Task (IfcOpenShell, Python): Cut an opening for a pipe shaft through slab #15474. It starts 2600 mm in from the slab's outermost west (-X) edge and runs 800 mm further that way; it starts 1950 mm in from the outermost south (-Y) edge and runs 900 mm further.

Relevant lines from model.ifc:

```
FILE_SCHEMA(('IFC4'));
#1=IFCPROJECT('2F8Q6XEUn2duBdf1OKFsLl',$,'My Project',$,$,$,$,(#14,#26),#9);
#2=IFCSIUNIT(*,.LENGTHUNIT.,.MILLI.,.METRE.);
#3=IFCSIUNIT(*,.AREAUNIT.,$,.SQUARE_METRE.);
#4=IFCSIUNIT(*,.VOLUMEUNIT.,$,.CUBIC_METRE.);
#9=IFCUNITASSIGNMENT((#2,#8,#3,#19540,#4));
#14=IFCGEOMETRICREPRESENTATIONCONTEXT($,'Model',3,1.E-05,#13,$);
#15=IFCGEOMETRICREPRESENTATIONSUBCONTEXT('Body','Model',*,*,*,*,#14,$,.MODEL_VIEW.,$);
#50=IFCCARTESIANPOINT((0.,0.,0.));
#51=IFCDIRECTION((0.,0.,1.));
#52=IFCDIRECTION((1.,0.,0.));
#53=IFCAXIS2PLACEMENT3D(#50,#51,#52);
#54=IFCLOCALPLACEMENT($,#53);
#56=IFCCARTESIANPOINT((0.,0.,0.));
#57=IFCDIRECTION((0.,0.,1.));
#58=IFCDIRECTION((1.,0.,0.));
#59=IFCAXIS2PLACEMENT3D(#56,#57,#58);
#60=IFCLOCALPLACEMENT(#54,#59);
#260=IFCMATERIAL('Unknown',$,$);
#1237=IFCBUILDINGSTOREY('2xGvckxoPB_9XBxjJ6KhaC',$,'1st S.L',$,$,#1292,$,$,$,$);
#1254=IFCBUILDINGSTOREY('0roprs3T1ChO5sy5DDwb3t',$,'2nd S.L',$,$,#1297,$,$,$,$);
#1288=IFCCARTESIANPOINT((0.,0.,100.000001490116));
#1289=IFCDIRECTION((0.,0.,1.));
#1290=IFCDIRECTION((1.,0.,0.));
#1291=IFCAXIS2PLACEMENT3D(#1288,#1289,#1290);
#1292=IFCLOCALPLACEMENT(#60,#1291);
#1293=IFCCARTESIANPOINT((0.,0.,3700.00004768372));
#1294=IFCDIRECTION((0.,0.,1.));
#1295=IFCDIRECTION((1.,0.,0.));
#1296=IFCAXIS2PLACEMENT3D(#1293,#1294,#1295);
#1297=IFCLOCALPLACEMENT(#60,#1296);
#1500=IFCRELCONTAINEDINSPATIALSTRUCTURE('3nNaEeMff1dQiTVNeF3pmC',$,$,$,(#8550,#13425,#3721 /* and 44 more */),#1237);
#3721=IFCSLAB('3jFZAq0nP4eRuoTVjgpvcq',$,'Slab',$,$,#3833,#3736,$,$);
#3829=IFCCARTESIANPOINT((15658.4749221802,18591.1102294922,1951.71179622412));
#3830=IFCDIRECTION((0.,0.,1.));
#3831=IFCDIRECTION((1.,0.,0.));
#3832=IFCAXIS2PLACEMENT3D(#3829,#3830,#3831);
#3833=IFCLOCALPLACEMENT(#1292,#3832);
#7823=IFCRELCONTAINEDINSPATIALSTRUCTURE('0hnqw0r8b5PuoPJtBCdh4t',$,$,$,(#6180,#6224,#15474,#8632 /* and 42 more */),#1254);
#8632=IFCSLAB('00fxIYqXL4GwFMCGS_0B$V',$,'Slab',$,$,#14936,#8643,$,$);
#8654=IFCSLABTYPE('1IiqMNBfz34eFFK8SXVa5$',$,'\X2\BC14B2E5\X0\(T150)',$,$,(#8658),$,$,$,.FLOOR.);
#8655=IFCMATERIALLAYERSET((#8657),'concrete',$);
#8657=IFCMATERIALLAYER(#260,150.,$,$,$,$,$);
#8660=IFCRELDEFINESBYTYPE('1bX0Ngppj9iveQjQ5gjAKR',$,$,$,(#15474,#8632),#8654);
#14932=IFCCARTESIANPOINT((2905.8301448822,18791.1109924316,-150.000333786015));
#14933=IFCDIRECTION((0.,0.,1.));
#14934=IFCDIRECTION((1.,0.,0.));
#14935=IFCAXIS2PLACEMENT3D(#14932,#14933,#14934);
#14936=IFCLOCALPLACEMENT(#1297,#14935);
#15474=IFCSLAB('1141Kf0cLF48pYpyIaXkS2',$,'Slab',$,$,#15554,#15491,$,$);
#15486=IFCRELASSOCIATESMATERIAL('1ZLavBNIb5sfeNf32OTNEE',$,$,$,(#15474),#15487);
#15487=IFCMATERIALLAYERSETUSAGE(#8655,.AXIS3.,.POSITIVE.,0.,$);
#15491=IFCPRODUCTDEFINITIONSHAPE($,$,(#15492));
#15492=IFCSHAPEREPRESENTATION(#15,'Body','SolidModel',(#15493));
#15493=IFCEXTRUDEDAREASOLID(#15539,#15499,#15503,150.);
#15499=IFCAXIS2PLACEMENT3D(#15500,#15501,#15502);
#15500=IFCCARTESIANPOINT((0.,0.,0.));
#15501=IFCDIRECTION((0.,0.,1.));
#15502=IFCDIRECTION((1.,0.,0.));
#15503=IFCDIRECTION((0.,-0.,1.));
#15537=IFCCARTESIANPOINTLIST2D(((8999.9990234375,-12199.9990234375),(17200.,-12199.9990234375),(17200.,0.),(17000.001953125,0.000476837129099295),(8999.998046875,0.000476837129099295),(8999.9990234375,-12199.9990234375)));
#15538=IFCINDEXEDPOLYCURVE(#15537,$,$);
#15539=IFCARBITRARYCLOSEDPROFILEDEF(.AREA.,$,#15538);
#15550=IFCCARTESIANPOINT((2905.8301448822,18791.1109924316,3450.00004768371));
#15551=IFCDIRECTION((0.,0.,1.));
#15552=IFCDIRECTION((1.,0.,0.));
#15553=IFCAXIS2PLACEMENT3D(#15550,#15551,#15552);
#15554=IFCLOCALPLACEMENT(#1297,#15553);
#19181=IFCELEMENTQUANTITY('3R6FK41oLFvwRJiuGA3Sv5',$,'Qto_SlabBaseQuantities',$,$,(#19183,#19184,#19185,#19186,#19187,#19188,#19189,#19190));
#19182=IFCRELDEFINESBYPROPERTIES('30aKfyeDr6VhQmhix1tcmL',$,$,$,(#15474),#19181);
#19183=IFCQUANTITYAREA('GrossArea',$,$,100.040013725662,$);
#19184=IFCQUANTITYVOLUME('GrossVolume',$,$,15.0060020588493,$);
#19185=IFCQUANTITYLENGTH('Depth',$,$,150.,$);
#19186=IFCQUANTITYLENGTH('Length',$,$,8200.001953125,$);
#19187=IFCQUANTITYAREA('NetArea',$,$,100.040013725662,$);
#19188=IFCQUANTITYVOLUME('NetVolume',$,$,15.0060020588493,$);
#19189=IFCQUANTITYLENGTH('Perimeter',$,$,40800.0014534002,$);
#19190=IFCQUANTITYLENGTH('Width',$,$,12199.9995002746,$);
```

```python
import numpy as np
import ifcopenshell
import ifcopenshell.api.feature
import ifcopenshell.api.geometry
import ifcopenshell.api.pset
import ifcopenshell.api.root
import ifcopenshell.geom
import ifcopenshell.util.element
import ifcopenshell.util.placement
import ifcopenshell.util.representation
import ifcopenshell.util.shape
import ifcopenshell.util.unit

model = ifcopenshell.open("model.ifc")
unit_scale = ifcopenshell.util.unit.calculate_unit_scale(model)
area_scale = ifcopenshell.util.unit.calculate_unit_scale(model, "AREAUNIT")
volume_scale = ifcopenshell.util.unit.calculate_unit_scale(model, "VOLUMEUNIT")
settings = ifcopenshell.geom.settings()


def volume(element):
    """Net volume in cubic metres, openings subtracted."""
    shape = ifcopenshell.geom.create_shape(settings, element)
    return ifcopenshell.util.shape.get_volume(shape.geometry)


slab = model.by_guid("1141Kf0cLF48pYpyIaXkS2")
before = volume(slab)

# Extent in the slab's own axes, in metres. The edges named are its -X and -Y sides.
slab_shape = ifcopenshell.geom.create_shape(settings, slab)
vertices = ifcopenshell.util.shape.get_vertices(slab_shape.geometry)
x_min, y_min, bottom = vertices.min(axis=0)
top = vertices[:, 2].max()

opening = ifcopenshell.api.root.create_entity(model, ifc_class="IfcOpeningElement", name="Pipe shaft opening", predefined_type="OPENING")
context = ifcopenshell.util.representation.get_context(model, "Model", "Body", "MODEL_VIEW")
width, depth = 0.8, 0.9
outline = [(0.0, 0.0), (width, 0.0), (width, depth), (0.0, depth), (0.0, 0.0)]
# Overshoot both faces by 50 mm so the cut is clean.
shape = ifcopenshell.api.geometry.add_slab_representation(
    model, context=context, depth=top - bottom + 0.1, polyline=outline
)
ifcopenshell.api.geometry.assign_representation(model, product=opening, representation=shape)

matrix = ifcopenshell.util.placement.get_local_placement(slab.ObjectPlacement)
matrix[:, 3] = matrix @ np.append(np.array([x_min + 2.6, y_min + 1.95, bottom - 0.05]) / unit_scale, 1.0)
ifcopenshell.api.geometry.edit_object_placement(model, product=opening, matrix=matrix, is_si=False)
ifcopenshell.api.feature.add_feature(model, feature=opening, element=slab)

after = volume(slab)

# Update the slab's stored quantities.
qto = model.by_id(ifcopenshell.util.element.get_pset(slab, "Qto_SlabBaseQuantities", should_inherit=False)["id"])
ifcopenshell.api.pset.edit_qto(model, qto=qto, properties={
    "NetArea": after / (top - bottom) / area_scale,
    "NetVolume": after / volume_scale,
})

print(f"slab volume {before:.3f} -> {after:.3f} m3")

model.write("model-out.ifc")
```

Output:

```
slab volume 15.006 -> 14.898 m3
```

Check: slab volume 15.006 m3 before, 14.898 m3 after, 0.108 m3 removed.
